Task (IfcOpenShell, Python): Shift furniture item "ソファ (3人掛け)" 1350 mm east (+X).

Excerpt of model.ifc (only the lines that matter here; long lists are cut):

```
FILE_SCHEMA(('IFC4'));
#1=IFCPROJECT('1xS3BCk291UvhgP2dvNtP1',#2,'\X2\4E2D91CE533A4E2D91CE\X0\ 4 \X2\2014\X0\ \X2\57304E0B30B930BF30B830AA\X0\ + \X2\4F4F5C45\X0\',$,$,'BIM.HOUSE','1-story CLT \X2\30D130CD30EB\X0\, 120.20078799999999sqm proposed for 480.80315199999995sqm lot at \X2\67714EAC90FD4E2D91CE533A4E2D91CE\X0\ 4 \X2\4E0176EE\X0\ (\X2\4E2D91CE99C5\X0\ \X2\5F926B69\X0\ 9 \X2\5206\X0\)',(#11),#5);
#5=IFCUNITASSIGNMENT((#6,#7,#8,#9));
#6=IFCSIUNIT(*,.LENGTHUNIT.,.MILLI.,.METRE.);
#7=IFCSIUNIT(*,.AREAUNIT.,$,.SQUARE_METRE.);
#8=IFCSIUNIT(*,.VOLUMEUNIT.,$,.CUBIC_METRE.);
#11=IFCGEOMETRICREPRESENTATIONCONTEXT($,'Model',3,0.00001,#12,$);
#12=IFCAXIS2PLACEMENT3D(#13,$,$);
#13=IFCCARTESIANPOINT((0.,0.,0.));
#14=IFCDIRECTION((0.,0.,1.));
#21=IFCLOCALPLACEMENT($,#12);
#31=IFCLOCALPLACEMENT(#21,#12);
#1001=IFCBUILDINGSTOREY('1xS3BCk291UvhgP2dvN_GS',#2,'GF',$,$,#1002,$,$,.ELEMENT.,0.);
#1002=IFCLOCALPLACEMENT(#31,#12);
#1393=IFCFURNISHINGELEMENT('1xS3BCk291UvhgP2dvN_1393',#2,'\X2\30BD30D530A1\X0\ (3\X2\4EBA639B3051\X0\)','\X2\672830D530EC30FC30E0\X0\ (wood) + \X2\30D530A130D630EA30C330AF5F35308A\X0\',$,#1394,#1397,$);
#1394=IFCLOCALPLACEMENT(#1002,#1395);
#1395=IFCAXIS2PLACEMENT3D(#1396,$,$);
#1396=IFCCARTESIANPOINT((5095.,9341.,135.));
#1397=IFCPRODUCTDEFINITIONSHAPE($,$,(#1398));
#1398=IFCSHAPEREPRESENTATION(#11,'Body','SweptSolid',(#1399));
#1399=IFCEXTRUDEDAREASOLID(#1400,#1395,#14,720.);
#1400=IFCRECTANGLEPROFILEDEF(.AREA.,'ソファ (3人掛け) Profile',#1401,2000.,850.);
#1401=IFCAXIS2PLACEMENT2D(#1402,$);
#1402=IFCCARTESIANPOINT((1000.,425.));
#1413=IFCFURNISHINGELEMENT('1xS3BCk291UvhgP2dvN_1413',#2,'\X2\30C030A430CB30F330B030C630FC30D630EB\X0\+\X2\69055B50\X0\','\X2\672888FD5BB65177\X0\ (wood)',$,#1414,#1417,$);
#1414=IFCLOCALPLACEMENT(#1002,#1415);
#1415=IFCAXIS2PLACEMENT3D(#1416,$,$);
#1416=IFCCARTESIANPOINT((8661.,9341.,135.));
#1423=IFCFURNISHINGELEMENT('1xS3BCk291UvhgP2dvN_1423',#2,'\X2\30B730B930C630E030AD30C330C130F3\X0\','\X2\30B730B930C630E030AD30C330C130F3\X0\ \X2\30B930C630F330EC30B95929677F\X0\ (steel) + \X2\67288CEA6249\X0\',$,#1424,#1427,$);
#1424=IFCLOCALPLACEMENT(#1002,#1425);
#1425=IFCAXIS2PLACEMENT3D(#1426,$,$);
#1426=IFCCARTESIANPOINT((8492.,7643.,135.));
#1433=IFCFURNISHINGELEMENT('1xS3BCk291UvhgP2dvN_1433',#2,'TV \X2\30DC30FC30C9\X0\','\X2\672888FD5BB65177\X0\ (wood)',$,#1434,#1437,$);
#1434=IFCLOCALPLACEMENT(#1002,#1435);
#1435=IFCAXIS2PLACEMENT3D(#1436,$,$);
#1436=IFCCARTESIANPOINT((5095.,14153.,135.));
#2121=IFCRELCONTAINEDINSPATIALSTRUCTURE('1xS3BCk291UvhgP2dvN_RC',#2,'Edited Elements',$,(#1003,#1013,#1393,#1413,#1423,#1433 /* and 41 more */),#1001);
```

```python
import ifcopenshell
import ifcopenshell.api.geometry
import ifcopenshell.util.placement

model = ifcopenshell.open("model.ifc")

item = model.by_id(1393)
matrix = ifcopenshell.util.placement.get_local_placement(item.ObjectPlacement)
matrix[0, 3] += 1350.0
ifcopenshell.api.geometry.edit_object_placement(model, product=item, matrix=matrix, is_si=False)

print(ifcopenshell.util.placement.get_local_placement(item.ObjectPlacement).round(3) + 0.0)

model.write("model-out.ifc")
```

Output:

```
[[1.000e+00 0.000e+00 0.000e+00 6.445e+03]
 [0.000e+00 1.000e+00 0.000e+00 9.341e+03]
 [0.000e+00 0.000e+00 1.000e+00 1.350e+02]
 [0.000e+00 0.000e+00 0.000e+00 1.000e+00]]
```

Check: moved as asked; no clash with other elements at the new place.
